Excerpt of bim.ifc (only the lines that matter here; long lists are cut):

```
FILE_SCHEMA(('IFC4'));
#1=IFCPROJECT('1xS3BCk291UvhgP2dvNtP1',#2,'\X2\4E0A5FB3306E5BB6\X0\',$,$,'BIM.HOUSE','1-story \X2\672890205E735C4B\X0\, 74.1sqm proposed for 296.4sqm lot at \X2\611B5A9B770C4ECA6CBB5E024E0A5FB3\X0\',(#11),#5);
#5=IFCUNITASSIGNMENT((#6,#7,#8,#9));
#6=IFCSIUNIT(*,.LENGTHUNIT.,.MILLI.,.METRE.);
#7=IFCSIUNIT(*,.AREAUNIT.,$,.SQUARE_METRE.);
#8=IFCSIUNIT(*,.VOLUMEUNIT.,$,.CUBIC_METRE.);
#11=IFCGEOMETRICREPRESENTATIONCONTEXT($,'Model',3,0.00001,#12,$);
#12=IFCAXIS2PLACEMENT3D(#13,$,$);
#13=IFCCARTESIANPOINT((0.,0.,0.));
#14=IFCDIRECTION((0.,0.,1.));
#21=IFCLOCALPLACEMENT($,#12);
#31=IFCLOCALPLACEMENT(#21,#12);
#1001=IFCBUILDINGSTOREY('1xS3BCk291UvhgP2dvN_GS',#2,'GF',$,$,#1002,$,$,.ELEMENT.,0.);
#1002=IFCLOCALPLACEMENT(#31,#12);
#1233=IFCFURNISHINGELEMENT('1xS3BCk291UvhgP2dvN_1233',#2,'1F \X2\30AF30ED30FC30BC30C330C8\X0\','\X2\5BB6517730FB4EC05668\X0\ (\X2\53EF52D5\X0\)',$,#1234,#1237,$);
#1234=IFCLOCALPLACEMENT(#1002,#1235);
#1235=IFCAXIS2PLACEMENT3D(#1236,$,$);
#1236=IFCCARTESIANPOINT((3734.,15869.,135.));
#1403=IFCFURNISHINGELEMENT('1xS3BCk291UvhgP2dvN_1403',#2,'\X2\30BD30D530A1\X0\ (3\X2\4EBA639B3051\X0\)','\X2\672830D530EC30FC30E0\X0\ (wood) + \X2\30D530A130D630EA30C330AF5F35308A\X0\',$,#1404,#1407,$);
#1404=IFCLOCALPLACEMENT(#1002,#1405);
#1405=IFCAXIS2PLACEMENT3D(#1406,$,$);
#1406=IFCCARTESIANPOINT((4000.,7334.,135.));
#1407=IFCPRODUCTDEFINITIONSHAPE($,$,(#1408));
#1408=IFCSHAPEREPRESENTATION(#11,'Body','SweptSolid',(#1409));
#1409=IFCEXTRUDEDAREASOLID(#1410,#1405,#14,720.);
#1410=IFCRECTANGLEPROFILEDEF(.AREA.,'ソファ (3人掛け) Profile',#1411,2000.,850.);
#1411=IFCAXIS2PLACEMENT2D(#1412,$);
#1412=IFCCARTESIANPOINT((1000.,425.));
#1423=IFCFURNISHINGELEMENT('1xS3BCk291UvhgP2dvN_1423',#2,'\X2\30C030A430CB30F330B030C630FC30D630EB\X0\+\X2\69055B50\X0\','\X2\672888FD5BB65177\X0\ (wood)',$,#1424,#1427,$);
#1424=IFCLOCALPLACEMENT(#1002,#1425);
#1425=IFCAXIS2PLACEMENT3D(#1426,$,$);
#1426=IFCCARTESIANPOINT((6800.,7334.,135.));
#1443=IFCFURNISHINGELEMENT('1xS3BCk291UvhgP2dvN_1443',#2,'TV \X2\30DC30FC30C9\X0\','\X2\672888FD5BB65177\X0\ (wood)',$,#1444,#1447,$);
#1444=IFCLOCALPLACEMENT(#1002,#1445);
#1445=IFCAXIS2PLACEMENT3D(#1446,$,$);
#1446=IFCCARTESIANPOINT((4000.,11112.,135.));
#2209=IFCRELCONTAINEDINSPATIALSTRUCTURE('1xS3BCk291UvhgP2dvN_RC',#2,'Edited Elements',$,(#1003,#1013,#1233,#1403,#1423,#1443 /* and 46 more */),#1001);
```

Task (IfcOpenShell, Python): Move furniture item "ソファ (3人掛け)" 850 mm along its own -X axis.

```python
import ifcopenshell
import ifcopenshell.api.geometry
import ifcopenshell.util.placement
import ifcopenshell.util.unit

model = ifcopenshell.open("bim.ifc")
unit_scale = ifcopenshell.util.unit.calculate_unit_scale(model)

item = model.by_id(1403)
matrix = ifcopenshell.util.placement.get_local_placement(item.ObjectPlacement)
matrix[:3, 3] -= matrix[:3, 0] * 0.85 / unit_scale
ifcopenshell.api.geometry.edit_object_placement(model, product=item, matrix=matrix, is_si=False)

print(ifcopenshell.util.placement.get_local_placement(item.ObjectPlacement).round(3) + 0.0)

model.write("bim_updated.ifc")
```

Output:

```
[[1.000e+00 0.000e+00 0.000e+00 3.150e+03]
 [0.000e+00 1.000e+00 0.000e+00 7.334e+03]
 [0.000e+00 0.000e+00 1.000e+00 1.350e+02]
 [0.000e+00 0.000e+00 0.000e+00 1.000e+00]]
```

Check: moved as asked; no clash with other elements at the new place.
